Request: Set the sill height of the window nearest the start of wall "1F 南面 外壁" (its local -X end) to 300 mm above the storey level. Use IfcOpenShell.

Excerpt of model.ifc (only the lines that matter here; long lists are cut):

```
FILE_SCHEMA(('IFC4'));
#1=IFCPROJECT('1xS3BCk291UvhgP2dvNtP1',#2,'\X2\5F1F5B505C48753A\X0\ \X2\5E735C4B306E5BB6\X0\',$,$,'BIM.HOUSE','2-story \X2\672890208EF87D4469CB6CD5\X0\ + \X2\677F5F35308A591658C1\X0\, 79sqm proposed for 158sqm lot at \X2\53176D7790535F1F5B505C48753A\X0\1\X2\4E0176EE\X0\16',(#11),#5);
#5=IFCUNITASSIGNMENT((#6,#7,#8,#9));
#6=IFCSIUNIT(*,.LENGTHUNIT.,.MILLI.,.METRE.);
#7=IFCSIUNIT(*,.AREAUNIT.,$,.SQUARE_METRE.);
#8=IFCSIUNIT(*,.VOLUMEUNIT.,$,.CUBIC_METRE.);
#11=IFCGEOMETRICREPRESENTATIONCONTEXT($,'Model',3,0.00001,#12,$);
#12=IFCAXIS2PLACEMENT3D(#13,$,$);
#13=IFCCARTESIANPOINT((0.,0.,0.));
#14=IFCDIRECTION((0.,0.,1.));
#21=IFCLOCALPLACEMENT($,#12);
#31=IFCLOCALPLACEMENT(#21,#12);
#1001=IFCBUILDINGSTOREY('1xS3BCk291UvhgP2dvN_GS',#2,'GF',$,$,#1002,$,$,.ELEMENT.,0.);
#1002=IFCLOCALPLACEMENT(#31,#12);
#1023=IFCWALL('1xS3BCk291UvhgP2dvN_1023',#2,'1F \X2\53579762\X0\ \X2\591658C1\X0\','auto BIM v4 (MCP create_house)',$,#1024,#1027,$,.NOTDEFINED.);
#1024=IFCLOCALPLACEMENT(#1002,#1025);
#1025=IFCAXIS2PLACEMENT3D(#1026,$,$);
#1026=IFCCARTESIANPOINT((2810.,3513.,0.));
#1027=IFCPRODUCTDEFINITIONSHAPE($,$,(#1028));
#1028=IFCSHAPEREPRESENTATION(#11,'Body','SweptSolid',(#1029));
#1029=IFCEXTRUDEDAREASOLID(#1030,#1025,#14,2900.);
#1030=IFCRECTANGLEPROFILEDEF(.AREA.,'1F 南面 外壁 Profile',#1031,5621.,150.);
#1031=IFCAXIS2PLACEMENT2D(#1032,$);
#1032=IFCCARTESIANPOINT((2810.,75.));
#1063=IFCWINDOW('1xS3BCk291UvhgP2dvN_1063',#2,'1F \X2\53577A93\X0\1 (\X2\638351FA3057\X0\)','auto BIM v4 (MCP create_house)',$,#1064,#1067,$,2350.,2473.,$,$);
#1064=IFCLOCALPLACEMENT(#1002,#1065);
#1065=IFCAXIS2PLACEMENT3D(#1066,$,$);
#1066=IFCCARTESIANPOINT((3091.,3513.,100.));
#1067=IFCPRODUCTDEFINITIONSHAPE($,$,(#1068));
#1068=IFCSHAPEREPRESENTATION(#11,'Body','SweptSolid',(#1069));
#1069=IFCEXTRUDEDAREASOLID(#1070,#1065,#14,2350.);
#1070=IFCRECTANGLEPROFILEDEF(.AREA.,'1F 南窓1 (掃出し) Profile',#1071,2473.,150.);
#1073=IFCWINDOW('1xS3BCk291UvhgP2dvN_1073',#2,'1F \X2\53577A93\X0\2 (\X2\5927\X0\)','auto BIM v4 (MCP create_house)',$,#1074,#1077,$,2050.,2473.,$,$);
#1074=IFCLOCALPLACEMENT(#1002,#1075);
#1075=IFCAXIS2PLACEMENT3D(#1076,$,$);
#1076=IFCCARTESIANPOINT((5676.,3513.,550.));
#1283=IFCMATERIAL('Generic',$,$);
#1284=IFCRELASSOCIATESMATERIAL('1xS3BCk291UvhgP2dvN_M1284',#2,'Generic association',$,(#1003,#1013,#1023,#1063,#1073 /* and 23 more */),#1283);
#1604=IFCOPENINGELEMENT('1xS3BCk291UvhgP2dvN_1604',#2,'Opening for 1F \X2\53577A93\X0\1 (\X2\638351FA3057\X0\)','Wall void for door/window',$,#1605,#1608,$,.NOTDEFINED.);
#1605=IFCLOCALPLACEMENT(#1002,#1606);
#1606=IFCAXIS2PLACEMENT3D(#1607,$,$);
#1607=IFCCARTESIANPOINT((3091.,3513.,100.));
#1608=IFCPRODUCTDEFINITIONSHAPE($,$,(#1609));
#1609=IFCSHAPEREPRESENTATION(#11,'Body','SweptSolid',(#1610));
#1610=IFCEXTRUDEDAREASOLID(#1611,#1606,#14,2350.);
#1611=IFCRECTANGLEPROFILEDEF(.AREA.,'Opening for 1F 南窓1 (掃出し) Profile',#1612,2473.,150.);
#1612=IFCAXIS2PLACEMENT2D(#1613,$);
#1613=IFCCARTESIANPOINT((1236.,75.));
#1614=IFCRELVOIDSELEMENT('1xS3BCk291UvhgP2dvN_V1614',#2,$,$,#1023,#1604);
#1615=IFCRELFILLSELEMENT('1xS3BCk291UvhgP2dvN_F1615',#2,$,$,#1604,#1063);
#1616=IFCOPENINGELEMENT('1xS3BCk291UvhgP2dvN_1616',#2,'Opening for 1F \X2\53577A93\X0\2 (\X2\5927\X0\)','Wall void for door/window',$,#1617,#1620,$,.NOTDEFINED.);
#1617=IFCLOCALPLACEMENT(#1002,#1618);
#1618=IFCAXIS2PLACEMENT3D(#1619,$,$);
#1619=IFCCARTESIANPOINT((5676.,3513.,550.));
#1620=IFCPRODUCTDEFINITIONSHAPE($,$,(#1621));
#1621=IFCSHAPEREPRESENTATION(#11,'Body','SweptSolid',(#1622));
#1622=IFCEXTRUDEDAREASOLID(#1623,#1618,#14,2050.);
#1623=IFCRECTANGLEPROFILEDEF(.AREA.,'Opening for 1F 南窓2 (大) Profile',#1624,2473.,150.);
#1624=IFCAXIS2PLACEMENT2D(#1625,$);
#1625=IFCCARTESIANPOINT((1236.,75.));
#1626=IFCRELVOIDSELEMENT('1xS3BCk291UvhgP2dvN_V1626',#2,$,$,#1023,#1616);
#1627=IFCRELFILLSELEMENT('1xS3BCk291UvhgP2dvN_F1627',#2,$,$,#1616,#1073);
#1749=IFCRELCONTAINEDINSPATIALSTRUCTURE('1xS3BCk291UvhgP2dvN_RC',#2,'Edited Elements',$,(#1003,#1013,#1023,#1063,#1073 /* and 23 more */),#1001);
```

```python
import numpy as np
import ifcopenshell
import ifcopenshell.api.geometry
import ifcopenshell.geom
import ifcopenshell.util.element
import ifcopenshell.util.placement
import ifcopenshell.util.shape
import ifcopenshell.util.unit

model = ifcopenshell.open("model.ifc")
unit_scale = ifcopenshell.util.unit.calculate_unit_scale(model)

window = model.by_guid("1xS3BCk291UvhgP2dvN_1063")
opening = window.FillsVoids[0].RelatingOpeningElement
storey = ifcopenshell.util.element.get_container(window, ifc_class="IfcBuildingStorey")
level = ifcopenshell.util.placement.get_local_placement(storey.ObjectPlacement)[2, 3]

# The opening's origin need not be at the sill, so measure its lowest point.
shape = ifcopenshell.geom.create_shape(ifcopenshell.geom.settings(), opening)
bottom = ifcopenshell.util.shape.get_shape_bottom_elevation(shape, shape.geometry) / unit_scale
dz = level + 0.3 / unit_scale - bottom

shift = np.array([0.0, 0.0, dz])
# The window is not placed relative to its opening, so move both.
for product in (opening, window):
    matrix = ifcopenshell.util.placement.get_local_placement(product.ObjectPlacement)
    matrix[:3, 3] += shift
    ifcopenshell.api.geometry.edit_object_placement(model, product=product, matrix=matrix, is_si=False)

print(f"moved by {dz * unit_scale:+.3f} m")

model.write("model_v2.ifc")
```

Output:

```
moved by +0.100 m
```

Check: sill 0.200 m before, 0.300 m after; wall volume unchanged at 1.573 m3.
